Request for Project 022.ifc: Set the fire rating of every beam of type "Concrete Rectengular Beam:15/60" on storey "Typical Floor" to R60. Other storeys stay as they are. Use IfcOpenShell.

First a look at what the model holds.

```python
import ifcopenshell
import ifcopenshell.util.element

model = ifcopenshell.open("Project 022.ifc")
print(model.schema)
storey = next(s for s in model.by_type("IfcBuildingStorey") if s.Name == "Typical Floor")
beams = [e for e in ifcopenshell.util.element.get_decomposition(storey) if e.is_a("IfcBeam")]
seen = {}
for e in beams:
    element_type = ifcopenshell.util.element.get_type(e)
    key = (element_type.Name if element_type != e and element_type else None, ifcopenshell.util.element.get_pset(e, "Pset_BeamCommon", "FireRating"))
    seen[key] = seen.get(key, 0) + 1
for (name, value), count in sorted(seen.items(), key=str):
    print(count, "x", name, "|", value)
```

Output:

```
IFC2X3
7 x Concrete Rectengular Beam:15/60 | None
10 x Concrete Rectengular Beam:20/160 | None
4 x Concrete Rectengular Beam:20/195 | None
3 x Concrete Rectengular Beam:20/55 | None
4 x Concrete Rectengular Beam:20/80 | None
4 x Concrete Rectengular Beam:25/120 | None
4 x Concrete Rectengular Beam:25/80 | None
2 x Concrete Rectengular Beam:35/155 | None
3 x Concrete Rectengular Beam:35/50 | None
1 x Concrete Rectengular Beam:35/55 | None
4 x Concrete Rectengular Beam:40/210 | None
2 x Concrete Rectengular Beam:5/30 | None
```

```python
import ifcopenshell
import ifcopenshell.api.pset
import ifcopenshell.util.element

model = ifcopenshell.open("Project 022.ifc")

storey = next(s for s in model.by_type("IfcBuildingStorey") if s.Name == "Typical Floor")
beams = [e for e in ifcopenshell.util.element.get_decomposition(storey) if e.is_a("IfcBeam")]

count = 0
for e in beams:
    element_type = ifcopenshell.util.element.get_type(e)
    if element_type in (None, e) or element_type.Name != "Concrete Rectengular Beam:15/60":
        continue
    # add_pset returns the element's existing set when there is one.
    pset = ifcopenshell.api.pset.add_pset(model, product=e, name="Pset_BeamCommon")
    ifcopenshell.api.pset.edit_pset(model, pset=pset, properties={"FireRating": "R60"})
    count += 1

print(count, "beams updated")

model.write("Project 022_rev.ifc")
```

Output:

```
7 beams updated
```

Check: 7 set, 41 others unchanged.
